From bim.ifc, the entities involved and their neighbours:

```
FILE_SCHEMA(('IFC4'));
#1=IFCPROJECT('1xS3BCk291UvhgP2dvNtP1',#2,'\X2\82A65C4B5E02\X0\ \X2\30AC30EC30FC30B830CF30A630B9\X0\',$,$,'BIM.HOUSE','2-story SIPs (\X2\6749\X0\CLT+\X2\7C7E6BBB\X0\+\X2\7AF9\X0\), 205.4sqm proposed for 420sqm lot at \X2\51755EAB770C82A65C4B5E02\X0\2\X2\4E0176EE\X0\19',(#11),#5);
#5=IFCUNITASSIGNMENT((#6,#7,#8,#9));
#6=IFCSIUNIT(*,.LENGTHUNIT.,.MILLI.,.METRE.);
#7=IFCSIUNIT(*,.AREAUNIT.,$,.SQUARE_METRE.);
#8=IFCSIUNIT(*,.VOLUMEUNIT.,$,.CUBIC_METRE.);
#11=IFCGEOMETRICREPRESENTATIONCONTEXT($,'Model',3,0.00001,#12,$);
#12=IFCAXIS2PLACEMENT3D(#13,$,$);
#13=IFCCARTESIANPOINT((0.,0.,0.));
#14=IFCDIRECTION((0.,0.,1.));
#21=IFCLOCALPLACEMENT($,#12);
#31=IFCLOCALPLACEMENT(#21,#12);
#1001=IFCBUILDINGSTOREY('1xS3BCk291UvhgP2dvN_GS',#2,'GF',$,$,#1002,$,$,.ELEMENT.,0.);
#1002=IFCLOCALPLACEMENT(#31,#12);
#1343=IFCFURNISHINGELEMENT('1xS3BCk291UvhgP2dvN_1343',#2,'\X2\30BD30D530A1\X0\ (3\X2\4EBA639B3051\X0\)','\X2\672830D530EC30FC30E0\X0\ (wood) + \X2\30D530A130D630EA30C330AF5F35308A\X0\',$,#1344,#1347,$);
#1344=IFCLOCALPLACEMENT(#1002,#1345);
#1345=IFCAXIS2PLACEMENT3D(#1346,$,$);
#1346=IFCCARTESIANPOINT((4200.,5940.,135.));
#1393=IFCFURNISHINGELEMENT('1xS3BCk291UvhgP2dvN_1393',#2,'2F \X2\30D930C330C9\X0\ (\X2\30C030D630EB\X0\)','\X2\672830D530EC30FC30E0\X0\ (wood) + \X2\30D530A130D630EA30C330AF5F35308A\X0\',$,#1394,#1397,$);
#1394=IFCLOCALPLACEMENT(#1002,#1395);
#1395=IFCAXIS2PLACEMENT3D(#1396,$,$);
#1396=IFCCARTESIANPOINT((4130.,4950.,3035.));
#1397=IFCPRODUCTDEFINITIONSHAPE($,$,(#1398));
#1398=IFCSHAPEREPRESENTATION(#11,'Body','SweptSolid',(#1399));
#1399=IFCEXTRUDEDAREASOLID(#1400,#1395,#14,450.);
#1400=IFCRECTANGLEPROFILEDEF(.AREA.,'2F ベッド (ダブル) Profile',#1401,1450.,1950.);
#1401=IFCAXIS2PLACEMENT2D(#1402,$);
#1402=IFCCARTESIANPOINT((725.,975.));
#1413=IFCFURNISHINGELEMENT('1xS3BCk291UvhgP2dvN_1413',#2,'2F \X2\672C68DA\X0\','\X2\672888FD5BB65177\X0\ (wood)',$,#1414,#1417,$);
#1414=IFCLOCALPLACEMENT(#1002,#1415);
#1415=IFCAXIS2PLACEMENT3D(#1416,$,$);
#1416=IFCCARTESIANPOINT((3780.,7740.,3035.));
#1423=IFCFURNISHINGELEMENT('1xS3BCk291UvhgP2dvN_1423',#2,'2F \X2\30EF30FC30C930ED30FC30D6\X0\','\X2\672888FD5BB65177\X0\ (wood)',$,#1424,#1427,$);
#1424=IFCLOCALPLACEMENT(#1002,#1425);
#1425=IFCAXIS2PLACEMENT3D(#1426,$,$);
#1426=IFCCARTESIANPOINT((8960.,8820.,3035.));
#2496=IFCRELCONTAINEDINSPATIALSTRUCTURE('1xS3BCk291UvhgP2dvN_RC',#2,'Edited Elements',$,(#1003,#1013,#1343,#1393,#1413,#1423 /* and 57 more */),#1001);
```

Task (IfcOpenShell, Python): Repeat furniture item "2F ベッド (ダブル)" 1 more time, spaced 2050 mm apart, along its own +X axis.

```python
import ifcopenshell
import ifcopenshell.api.geometry
import ifcopenshell.api.root
import ifcopenshell.util.element
import ifcopenshell.util.placement
import ifcopenshell.util.unit

model = ifcopenshell.open("bim.ifc")
unit_scale = ifcopenshell.util.unit.calculate_unit_scale(model)


def reuse_history(source, copy):
    """copy_class also copies each property set's owner history, people and application; keep the originals."""
    for rel in copy.IsDefinedBy:
        if rel.is_a("IfcRelDefinesByProperties") and (history := rel.RelatingPropertyDefinition.OwnerHistory):
            rel.RelatingPropertyDefinition.OwnerHistory = source.OwnerHistory
            ifcopenshell.util.element.remove_deep2(model, history)


source = model.by_guid("1xS3BCk291UvhgP2dvN_1393")
base = ifcopenshell.util.placement.get_local_placement(source.ObjectPlacement)
step = base[:3, 0] * 2.05 / unit_scale

for i in range(1, 2):
    copy = ifcopenshell.api.root.copy_class(model, product=source)
    copy.Representation = ifcopenshell.util.element.copy_deep(
        model, source.Representation, exclude=["IfcGeometricRepresentationContext", "IfcRepresentationMap"]
    )
    reuse_history(source, copy)
    matrix = base.copy()
    matrix[:3, 3] += i * step
    print("added at", matrix[:3, 3].round(3) + 0.0)
    ifcopenshell.api.geometry.edit_object_placement(model, product=copy, matrix=matrix, is_si=False)

model.write("bim_v2.ifc")
```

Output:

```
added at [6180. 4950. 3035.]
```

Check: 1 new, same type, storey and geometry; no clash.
